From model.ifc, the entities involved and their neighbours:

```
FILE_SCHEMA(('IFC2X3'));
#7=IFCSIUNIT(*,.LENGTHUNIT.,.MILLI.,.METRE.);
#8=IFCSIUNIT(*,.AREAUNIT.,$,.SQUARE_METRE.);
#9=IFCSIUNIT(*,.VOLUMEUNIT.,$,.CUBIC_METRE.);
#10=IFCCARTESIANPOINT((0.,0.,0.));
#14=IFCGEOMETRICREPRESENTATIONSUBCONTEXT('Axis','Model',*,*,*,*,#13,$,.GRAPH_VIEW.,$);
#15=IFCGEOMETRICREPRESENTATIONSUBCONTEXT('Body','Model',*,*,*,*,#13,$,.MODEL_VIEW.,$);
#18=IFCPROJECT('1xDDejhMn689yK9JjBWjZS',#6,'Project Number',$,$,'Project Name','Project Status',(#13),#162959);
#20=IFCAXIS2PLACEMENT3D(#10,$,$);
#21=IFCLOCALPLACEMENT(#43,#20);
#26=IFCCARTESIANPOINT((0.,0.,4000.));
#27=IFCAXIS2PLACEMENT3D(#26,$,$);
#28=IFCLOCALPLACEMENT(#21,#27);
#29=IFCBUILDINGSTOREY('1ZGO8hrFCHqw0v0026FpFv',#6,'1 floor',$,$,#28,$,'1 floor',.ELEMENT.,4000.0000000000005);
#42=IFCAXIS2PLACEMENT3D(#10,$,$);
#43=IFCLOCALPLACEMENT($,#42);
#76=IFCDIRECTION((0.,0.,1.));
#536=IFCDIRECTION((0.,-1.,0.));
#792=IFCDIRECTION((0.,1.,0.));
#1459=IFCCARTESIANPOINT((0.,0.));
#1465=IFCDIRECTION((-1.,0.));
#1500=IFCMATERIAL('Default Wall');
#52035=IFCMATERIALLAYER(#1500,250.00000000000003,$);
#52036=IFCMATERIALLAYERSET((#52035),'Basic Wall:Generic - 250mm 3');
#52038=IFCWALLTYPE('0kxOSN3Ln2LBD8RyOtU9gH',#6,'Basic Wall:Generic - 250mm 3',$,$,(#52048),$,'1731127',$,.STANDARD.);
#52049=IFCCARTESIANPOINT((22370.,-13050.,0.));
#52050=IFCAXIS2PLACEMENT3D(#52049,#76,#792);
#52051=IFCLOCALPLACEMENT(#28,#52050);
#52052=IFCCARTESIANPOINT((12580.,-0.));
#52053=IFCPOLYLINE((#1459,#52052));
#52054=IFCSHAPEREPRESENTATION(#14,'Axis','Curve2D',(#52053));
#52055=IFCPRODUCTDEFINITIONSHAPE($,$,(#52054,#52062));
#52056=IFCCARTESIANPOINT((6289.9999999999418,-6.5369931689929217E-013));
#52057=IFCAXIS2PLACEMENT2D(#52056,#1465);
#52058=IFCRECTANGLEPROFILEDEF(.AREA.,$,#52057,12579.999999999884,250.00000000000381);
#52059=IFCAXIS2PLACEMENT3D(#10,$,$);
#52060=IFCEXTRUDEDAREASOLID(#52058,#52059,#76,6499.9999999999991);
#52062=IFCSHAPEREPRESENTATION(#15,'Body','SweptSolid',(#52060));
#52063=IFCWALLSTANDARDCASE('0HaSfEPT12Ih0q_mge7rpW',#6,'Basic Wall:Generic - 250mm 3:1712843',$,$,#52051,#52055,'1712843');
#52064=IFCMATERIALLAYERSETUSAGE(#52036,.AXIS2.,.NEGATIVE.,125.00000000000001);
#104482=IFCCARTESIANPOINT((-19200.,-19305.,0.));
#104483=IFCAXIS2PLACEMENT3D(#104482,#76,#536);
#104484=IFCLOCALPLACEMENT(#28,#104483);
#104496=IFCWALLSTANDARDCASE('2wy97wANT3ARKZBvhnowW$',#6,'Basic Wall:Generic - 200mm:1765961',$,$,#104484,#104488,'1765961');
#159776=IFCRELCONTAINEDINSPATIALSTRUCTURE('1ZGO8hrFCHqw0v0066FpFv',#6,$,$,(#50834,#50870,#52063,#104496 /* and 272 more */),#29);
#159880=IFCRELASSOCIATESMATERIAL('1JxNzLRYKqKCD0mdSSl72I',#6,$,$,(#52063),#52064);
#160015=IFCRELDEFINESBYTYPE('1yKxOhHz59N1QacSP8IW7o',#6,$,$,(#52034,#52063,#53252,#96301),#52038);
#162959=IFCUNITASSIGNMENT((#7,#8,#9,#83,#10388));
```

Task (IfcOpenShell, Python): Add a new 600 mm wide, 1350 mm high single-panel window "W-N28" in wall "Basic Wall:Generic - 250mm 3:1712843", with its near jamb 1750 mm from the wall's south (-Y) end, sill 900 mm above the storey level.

```python
import numpy as np
import ifcopenshell
import ifcopenshell.api.feature
import ifcopenshell.api.geometry
import ifcopenshell.api.root
import ifcopenshell.api.spatial
import ifcopenshell.api.type
import ifcopenshell.geom
import ifcopenshell.util.element
import ifcopenshell.util.placement
import ifcopenshell.util.representation
import ifcopenshell.util.shape
import ifcopenshell.util.unit

model = ifcopenshell.open("model.ifc")
unit_scale = ifcopenshell.util.unit.calculate_unit_scale(model)
settings = ifcopenshell.geom.settings()


def volume(element):
    """Net volume in cubic metres, openings subtracted."""
    shape = ifcopenshell.geom.create_shape(settings, element)
    return ifcopenshell.util.shape.get_volume(shape.geometry)


wall = model.by_guid("0HaSfEPT12Ih0q_mge7rpW")
storey = ifcopenshell.util.element.get_container(wall, ifc_class="IfcBuildingStorey")
context = ifcopenshell.util.representation.get_context(model, "Model", "Body", "MODEL_VIEW")
before = volume(wall)

width, height, from_end, sill = 0.6, 1.35, 1.75, 0.9  # metres

# The wall runs along its own X axis, and the end named is its -X end.
wall_shape = ifcopenshell.geom.create_shape(settings, wall)
x, y, z = ifcopenshell.util.shape.get_vertices(wall_shape.geometry).T
start = x.min() + from_end
face, thickness = float(y.min()), float(y.max() - y.min())
wall_matrix = ifcopenshell.util.placement.get_local_placement(wall.ObjectPlacement)
level = ifcopenshell.util.placement.get_local_placement(storey.ObjectPlacement)[2, 3]


def in_wall(x, y):
    """Placement at x, y metres in the wall's axes, at sill height."""
    matrix = wall_matrix.copy()
    matrix[:, 3] = wall_matrix @ np.array([x / unit_scale, y / unit_scale, 0.0, 1.0])
    matrix[2, 3] = level + sill / unit_scale
    return matrix


# Opening: a box that overshoots both wall faces by 50 mm.
opening = ifcopenshell.api.root.create_entity(model, ifc_class="IfcOpeningElement")
box = ifcopenshell.api.geometry.add_wall_representation(
    model, context=context, length=width, height=height, thickness=thickness + 0.1
)
ifcopenshell.api.geometry.assign_representation(model, product=opening, representation=box)
ifcopenshell.api.geometry.edit_object_placement(model, product=opening, matrix=in_wall(start, face - 0.05), is_si=False)
ifcopenshell.api.feature.add_feature(model, feature=opening, element=wall)

window = ifcopenshell.api.root.create_entity(model, ifc_class="IfcWindow", name="W-N28")
window.OverallWidth, window.OverallHeight = width / unit_scale, height / unit_scale
body = ifcopenshell.api.geometry.add_window_representation(
    model,
    context=context,
    overall_width=window.OverallWidth,
    overall_height=window.OverallHeight,
    partition_type="SINGLE_PANEL",
)
ifcopenshell.api.geometry.assign_representation(model, product=window, representation=body)
ifcopenshell.api.spatial.assign_container(model, products=[window], relating_structure=storey)
fills = ifcopenshell.api.feature.add_filling(model, opening=opening, element=window)
fills.OwnerHistory = window.OwnerHistory  # required in IFC2X3

# IFC2X3 keeps the operation on the window style.
style = ifcopenshell.api.root.create_entity(model, ifc_class="IfcWindowStyle", name="W-N28")
style.OperationType, style.ConstructionType = "SINGLE_PANEL", "NOTDEFINED"
style.ParameterTakesPrecedence = style.Sizeable = False
ifcopenshell.api.type.assign_type(model, related_objects=[window], relating_type=style)

# Centre the window in the wall's thickness.
ifcopenshell.api.geometry.edit_object_placement(model, product=window, matrix=in_wall(start, face), is_si=False)
window_shape = ifcopenshell.geom.create_shape(settings, window)
depth = ifcopenshell.util.shape.get_vertices(window_shape.geometry)[:, 1]
offset = face + thickness / 2 - (depth.min() + depth.max()) / 2
ifcopenshell.api.geometry.edit_object_placement(model, product=window, matrix=in_wall(start, offset), is_si=False)

after = volume(wall)

print(f"wall volume {before:.3f} -> {after:.3f} m3")

model.write("model-out.ifc")
```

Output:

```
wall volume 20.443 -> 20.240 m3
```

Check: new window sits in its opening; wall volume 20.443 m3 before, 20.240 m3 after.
